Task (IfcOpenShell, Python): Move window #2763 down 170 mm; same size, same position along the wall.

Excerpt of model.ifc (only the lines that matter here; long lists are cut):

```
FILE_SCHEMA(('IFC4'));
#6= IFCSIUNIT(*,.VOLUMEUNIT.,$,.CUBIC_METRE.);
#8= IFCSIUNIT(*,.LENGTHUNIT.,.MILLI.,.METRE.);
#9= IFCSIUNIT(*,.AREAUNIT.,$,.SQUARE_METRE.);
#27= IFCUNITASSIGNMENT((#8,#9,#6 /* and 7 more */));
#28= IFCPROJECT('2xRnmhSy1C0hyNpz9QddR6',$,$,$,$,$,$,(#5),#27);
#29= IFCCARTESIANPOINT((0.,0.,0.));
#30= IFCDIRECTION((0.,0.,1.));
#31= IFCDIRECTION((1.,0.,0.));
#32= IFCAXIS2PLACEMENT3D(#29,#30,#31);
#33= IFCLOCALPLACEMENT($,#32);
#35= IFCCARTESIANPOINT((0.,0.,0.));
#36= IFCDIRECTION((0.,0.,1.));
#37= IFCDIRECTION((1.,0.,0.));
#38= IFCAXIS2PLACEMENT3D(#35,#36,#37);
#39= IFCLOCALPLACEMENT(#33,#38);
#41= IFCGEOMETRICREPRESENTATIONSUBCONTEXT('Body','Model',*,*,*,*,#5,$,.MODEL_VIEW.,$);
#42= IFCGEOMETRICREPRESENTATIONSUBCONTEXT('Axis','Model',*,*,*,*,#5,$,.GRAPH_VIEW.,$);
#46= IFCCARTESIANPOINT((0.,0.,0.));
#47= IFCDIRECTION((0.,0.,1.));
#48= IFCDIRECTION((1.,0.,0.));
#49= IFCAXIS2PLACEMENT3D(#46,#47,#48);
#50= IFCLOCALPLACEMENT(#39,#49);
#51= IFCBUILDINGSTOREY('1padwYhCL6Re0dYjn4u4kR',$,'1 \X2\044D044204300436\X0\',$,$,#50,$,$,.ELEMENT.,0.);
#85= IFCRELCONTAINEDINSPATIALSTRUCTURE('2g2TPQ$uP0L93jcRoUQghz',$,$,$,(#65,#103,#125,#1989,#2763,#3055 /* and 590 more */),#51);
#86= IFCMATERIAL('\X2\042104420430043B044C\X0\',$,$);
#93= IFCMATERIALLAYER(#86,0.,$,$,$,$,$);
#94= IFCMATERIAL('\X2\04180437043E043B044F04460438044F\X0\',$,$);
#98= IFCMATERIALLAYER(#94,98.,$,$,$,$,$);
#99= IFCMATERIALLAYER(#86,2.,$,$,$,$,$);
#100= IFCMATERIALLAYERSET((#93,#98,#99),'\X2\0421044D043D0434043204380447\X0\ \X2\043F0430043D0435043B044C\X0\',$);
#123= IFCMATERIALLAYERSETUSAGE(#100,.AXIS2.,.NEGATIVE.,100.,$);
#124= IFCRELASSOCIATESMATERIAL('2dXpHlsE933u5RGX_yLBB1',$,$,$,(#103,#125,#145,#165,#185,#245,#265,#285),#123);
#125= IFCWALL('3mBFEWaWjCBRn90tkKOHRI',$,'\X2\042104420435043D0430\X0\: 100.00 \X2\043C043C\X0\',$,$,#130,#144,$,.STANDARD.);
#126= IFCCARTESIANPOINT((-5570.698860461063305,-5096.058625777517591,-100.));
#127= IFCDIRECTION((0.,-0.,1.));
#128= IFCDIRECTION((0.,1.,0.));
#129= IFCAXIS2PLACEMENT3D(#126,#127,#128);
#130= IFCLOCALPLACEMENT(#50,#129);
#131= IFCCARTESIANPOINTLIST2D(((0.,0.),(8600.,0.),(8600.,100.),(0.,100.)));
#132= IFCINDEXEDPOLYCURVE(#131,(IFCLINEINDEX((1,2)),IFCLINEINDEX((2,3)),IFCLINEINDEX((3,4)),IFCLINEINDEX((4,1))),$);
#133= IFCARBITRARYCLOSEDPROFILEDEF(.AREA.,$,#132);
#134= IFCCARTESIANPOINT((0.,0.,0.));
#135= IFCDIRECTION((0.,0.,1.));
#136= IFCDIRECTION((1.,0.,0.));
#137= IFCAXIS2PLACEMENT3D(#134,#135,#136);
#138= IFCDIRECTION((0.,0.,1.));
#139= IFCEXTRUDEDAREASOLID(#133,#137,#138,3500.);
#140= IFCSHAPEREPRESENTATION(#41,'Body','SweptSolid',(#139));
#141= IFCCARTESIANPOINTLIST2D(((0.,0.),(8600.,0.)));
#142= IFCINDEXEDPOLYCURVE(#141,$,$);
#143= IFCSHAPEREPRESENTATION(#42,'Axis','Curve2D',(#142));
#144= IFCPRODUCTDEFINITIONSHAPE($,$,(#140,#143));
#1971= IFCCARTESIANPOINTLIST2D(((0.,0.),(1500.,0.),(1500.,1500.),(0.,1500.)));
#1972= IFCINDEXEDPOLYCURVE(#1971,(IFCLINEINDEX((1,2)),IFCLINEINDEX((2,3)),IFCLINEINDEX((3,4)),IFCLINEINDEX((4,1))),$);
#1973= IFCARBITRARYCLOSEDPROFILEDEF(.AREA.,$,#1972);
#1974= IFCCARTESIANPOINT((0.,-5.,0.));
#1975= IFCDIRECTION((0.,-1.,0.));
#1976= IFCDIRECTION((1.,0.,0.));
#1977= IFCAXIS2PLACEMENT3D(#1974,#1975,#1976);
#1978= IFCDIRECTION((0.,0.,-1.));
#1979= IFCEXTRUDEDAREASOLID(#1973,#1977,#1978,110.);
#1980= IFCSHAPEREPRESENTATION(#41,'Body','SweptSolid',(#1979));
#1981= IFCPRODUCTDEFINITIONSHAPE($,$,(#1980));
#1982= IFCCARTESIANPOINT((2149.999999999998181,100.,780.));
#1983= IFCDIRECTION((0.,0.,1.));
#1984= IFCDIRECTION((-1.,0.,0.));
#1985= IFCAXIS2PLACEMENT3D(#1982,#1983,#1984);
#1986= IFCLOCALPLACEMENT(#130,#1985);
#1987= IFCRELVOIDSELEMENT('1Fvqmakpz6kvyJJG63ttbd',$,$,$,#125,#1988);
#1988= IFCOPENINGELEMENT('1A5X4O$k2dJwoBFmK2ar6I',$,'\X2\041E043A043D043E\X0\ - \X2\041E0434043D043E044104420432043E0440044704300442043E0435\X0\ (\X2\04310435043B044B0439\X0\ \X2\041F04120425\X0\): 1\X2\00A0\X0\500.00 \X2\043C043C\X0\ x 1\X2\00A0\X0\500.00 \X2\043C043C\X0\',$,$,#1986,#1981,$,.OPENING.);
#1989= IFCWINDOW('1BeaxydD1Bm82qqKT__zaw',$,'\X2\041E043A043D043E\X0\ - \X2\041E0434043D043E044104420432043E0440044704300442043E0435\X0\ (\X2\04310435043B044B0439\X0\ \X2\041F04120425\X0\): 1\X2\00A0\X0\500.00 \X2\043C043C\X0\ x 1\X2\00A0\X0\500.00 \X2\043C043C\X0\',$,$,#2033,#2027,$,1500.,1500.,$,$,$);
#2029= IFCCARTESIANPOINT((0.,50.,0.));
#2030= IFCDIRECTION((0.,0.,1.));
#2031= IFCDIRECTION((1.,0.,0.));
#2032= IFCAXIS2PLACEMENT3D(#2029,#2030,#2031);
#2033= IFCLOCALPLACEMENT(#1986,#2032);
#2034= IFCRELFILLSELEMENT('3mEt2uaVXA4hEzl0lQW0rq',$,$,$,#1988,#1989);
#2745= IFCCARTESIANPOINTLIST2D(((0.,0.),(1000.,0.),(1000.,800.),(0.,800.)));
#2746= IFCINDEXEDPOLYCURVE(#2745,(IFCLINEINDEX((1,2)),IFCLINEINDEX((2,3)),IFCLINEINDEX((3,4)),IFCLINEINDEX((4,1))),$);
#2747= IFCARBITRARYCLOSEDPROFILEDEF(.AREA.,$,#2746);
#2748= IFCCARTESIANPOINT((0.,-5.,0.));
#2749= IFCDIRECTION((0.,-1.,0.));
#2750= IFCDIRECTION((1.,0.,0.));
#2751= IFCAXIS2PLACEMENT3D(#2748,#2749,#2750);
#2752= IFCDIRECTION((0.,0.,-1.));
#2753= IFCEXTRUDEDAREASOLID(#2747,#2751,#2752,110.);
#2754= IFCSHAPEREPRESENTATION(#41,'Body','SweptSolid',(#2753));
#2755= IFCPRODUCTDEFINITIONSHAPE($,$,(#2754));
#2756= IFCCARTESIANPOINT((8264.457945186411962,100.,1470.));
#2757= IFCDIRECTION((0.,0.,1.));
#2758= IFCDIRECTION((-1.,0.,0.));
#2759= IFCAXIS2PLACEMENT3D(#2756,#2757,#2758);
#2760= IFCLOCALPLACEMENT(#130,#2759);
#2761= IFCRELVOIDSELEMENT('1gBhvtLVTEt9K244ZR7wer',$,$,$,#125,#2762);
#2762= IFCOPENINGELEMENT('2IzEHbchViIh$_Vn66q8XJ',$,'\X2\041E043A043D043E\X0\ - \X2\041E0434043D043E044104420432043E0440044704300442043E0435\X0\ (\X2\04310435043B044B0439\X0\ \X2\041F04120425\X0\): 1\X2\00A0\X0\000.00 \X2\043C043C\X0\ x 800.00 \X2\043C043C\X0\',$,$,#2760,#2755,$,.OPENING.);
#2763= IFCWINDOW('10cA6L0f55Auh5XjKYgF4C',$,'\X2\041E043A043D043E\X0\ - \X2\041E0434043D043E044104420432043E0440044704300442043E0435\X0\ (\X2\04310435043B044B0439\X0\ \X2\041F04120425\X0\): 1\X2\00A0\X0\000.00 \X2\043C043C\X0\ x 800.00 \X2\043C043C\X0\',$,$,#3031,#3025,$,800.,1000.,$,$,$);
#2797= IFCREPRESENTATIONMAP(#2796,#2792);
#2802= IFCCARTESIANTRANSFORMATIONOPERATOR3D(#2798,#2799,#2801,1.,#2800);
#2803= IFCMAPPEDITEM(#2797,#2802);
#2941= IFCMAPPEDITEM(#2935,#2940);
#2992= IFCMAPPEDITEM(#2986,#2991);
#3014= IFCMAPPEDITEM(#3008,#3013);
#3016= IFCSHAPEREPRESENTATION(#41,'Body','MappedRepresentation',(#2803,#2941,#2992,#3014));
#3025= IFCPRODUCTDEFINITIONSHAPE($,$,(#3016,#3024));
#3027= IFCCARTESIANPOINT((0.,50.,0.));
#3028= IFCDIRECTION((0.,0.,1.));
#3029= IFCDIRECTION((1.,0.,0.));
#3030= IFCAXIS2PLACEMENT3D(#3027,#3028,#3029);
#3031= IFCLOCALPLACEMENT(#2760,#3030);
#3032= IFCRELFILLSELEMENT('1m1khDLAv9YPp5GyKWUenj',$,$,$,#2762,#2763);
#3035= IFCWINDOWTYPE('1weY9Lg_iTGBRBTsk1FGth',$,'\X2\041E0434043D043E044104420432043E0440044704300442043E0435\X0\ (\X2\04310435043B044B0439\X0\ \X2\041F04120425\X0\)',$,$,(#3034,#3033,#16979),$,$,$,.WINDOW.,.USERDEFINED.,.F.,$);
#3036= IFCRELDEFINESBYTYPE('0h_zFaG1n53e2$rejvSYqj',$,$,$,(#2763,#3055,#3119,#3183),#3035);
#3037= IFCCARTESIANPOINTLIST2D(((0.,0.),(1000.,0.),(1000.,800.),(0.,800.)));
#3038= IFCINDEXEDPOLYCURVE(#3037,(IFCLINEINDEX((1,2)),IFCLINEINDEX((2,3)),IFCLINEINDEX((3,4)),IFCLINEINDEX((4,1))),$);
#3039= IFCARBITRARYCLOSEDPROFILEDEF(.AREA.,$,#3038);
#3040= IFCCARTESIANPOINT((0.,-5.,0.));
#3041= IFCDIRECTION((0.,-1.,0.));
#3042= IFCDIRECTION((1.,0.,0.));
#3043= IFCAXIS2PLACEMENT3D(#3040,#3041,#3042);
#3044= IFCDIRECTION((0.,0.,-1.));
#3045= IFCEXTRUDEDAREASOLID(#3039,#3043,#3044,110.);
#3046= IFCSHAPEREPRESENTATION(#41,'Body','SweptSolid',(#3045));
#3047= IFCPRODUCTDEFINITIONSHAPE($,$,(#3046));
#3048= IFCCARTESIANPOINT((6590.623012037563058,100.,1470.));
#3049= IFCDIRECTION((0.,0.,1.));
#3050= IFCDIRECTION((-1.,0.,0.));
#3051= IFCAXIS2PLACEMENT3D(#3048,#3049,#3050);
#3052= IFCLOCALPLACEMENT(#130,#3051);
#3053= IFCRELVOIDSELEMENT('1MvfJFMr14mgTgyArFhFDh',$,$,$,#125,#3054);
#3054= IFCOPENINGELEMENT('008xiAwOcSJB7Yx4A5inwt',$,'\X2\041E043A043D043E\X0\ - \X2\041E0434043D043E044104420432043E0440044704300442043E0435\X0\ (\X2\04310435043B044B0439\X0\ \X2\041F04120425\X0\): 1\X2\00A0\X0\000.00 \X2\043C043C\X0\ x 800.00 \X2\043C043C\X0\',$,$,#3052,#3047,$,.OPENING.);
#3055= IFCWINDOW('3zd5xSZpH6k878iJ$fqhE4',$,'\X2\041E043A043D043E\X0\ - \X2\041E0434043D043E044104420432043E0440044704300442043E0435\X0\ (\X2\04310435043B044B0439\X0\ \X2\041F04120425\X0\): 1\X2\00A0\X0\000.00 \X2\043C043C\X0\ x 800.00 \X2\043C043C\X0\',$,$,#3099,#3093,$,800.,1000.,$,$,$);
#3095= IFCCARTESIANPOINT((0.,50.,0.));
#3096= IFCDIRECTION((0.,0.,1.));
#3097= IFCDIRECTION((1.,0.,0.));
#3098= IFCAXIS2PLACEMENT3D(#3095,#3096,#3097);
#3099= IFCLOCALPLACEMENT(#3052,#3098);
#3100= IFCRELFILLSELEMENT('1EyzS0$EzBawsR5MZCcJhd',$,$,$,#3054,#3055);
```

```python
import numpy as np
import ifcopenshell
import ifcopenshell.api.geometry
import ifcopenshell.util.placement
import ifcopenshell.util.unit

model = ifcopenshell.open("model.ifc")
unit_scale = ifcopenshell.util.unit.calculate_unit_scale(model)

window = model.by_id(2763)
opening = window.FillsVoids[0].RelatingOpeningElement
dz = -0.17 / unit_scale

shift = np.array([0.0, 0.0, dz])
# The window is placed relative to its opening, so it follows when the opening moves.
matrix = ifcopenshell.util.placement.get_local_placement(opening.ObjectPlacement)
matrix[:3, 3] += shift
ifcopenshell.api.geometry.edit_object_placement(
    model, product=opening, matrix=matrix, is_si=False, should_transform_children=True
)

print(f"moved by {dz * unit_scale:+.3f} m")

model.write("model_v2.ifc")
```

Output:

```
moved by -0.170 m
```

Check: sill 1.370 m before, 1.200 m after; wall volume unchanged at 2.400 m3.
